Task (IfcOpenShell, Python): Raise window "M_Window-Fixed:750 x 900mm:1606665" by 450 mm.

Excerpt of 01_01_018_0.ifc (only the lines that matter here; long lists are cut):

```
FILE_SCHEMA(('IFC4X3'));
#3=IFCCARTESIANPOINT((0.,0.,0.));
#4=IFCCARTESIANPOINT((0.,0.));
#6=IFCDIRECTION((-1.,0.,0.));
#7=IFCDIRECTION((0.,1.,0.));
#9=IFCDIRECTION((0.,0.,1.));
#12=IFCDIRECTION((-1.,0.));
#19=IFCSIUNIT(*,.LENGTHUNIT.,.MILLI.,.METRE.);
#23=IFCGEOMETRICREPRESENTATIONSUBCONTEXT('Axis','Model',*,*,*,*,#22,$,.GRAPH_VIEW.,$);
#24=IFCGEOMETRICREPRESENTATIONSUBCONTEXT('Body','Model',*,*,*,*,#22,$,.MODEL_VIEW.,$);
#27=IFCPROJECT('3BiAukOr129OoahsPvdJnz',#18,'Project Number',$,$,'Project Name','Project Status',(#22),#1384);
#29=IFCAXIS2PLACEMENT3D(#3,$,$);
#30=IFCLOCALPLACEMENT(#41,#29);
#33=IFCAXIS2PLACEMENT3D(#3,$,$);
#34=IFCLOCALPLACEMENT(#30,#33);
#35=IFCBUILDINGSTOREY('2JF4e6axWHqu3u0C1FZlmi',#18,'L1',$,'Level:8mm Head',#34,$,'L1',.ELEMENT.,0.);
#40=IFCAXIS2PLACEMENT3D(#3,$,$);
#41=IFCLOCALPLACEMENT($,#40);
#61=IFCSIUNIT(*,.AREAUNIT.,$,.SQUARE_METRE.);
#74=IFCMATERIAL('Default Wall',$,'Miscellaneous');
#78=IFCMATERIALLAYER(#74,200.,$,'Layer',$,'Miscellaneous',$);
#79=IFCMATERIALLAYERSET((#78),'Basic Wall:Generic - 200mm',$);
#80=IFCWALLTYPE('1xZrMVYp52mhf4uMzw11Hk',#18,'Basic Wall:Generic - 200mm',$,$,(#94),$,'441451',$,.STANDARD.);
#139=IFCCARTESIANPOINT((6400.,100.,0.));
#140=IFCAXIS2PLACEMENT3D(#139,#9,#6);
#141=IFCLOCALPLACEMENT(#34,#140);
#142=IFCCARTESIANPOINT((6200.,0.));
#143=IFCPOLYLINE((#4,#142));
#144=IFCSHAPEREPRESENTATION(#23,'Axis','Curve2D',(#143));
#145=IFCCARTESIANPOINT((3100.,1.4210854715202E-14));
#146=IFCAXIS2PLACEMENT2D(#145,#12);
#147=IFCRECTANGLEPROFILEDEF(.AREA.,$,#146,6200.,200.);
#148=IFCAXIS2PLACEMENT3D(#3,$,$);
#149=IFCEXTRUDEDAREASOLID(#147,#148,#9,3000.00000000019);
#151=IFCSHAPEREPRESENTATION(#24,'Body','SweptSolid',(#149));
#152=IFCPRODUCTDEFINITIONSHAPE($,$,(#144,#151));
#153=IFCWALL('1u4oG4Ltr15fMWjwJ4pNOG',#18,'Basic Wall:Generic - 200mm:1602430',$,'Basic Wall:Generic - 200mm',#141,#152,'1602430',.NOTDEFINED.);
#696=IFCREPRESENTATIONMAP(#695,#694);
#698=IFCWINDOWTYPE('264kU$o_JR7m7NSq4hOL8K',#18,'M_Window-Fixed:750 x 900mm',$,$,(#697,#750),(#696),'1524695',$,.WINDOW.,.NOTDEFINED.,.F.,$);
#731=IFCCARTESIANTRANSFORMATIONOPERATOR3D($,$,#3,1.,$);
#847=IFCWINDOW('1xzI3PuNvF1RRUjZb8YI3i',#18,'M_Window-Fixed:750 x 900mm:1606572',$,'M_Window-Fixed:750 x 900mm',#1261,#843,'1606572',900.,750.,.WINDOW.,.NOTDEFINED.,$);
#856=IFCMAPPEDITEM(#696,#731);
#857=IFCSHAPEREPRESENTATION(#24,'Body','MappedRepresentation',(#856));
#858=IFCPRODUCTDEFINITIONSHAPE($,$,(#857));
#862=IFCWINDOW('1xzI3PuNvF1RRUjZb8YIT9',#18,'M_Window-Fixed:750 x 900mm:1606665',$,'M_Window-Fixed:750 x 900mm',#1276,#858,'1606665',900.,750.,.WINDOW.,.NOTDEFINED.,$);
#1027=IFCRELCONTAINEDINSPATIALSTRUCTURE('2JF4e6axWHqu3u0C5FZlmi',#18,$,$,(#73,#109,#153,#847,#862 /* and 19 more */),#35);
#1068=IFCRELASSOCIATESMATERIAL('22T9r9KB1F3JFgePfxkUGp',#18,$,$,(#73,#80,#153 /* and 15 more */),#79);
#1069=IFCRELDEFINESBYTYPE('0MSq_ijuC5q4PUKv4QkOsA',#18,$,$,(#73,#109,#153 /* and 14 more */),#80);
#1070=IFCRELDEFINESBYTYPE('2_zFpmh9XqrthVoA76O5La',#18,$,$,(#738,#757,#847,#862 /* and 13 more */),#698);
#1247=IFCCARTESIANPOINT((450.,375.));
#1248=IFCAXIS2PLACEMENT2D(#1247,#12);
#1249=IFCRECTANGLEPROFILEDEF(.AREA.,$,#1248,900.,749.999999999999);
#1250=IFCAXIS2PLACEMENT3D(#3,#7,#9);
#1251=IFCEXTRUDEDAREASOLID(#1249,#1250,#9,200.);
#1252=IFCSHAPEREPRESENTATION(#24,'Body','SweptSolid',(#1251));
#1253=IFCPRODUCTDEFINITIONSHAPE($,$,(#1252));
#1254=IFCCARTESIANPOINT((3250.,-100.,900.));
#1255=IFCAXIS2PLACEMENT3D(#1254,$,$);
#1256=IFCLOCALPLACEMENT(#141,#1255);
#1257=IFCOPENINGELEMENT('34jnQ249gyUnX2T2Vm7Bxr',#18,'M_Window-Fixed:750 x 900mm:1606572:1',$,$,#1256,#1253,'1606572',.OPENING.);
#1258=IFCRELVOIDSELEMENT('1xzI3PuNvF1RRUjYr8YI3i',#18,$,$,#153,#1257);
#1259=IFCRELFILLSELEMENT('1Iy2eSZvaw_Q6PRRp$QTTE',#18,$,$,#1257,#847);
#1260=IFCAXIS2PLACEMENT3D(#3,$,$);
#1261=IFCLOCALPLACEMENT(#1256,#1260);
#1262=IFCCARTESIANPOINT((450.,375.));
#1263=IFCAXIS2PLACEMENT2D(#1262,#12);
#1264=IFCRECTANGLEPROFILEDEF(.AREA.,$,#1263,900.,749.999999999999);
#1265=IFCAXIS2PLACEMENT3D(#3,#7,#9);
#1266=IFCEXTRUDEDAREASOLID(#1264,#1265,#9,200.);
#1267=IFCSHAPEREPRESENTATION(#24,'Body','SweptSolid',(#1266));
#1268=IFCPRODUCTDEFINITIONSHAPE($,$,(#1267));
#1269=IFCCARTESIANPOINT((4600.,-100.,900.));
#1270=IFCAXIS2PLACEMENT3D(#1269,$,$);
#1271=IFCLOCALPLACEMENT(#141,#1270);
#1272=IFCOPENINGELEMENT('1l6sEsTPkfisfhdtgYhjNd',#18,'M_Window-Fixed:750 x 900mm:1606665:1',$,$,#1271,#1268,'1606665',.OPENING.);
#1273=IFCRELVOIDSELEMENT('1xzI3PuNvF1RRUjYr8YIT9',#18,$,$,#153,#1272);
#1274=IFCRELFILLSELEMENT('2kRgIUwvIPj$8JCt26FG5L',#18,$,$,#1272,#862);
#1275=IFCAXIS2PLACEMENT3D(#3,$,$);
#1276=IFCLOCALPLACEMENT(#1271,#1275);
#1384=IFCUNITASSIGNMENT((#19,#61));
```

```python
import numpy as np
import ifcopenshell
import ifcopenshell.api.geometry
import ifcopenshell.util.placement
import ifcopenshell.util.unit

model = ifcopenshell.open("01_01_018_0.ifc")
unit_scale = ifcopenshell.util.unit.calculate_unit_scale(model)

window = model.by_guid("1xzI3PuNvF1RRUjZb8YIT9")
opening = window.FillsVoids[0].RelatingOpeningElement
dz = 450.0

shift = np.array([0.0, 0.0, dz])
# The window is placed relative to its opening, so it follows when the opening moves.
matrix = ifcopenshell.util.placement.get_local_placement(opening.ObjectPlacement)
matrix[:3, 3] += shift
ifcopenshell.api.geometry.edit_object_placement(
    model, product=opening, matrix=matrix, is_si=False, should_transform_children=True
)

print(f"moved by {dz * unit_scale:+.3f} m")

model.write("01_01_018_0_v2.ifc")
```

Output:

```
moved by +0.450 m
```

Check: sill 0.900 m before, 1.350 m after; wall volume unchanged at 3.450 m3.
